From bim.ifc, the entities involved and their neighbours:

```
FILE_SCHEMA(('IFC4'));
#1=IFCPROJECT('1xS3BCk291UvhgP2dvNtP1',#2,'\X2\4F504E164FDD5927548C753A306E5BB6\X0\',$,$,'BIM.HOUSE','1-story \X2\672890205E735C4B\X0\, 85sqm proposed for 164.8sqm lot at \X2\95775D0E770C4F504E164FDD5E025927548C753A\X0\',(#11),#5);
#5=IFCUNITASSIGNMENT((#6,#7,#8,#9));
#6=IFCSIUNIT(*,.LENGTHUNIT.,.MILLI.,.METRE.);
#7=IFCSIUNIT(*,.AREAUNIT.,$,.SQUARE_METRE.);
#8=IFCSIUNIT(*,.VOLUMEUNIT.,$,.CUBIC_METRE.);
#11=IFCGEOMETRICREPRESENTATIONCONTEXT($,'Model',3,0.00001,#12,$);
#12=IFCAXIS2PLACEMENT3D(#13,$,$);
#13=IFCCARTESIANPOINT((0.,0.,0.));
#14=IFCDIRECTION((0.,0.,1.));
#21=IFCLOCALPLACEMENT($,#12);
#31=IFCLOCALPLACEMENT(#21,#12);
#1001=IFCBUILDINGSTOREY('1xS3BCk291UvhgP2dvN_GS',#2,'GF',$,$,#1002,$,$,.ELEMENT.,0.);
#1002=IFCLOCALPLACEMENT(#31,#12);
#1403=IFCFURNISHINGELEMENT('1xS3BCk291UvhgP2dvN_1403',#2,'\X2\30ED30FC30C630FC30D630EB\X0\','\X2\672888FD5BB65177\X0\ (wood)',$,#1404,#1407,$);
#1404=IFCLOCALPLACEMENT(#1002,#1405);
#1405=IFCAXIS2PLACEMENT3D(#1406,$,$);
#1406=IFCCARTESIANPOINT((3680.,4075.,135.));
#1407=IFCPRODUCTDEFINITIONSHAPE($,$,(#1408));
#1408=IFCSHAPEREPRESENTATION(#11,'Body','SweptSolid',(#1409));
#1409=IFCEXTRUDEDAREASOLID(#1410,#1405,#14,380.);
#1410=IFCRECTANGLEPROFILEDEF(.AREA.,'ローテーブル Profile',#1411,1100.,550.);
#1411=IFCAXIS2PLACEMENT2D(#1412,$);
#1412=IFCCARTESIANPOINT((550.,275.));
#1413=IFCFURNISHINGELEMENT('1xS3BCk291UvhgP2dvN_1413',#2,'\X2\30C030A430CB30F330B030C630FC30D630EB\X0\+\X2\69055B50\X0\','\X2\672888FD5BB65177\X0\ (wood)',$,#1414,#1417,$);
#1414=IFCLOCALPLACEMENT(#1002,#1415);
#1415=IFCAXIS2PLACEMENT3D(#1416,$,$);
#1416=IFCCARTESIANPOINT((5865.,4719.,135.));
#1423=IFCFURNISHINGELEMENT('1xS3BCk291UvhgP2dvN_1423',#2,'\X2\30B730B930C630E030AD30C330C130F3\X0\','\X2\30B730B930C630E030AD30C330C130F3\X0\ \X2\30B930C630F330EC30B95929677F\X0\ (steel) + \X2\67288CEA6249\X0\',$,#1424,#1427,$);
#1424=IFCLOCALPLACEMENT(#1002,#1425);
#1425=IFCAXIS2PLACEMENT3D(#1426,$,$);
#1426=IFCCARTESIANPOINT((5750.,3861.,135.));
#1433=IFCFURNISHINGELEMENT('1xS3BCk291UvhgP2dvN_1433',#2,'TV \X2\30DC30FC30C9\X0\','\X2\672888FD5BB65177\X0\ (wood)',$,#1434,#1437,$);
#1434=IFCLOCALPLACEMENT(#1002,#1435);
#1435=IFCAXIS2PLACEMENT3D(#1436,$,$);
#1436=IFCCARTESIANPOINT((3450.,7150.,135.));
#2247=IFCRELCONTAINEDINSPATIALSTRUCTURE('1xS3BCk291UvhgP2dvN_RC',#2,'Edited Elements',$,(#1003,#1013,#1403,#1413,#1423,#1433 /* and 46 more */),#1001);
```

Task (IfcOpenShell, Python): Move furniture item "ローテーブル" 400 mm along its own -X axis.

```python
import ifcopenshell
import ifcopenshell.api.geometry
import ifcopenshell.util.placement
import ifcopenshell.util.unit

model = ifcopenshell.open("bim.ifc")
unit_scale = ifcopenshell.util.unit.calculate_unit_scale(model)

item = model.by_id(1403)
matrix = ifcopenshell.util.placement.get_local_placement(item.ObjectPlacement)
matrix[:3, 3] -= matrix[:3, 0] * 0.4 / unit_scale
ifcopenshell.api.geometry.edit_object_placement(model, product=item, matrix=matrix, is_si=False)

print(ifcopenshell.util.placement.get_local_placement(item.ObjectPlacement).round(3) + 0.0)

model.write("bim_updated.ifc")
```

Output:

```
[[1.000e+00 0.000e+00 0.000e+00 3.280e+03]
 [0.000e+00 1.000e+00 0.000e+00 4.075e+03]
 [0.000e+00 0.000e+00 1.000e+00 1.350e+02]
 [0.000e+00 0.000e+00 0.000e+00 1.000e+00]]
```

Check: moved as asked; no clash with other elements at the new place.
